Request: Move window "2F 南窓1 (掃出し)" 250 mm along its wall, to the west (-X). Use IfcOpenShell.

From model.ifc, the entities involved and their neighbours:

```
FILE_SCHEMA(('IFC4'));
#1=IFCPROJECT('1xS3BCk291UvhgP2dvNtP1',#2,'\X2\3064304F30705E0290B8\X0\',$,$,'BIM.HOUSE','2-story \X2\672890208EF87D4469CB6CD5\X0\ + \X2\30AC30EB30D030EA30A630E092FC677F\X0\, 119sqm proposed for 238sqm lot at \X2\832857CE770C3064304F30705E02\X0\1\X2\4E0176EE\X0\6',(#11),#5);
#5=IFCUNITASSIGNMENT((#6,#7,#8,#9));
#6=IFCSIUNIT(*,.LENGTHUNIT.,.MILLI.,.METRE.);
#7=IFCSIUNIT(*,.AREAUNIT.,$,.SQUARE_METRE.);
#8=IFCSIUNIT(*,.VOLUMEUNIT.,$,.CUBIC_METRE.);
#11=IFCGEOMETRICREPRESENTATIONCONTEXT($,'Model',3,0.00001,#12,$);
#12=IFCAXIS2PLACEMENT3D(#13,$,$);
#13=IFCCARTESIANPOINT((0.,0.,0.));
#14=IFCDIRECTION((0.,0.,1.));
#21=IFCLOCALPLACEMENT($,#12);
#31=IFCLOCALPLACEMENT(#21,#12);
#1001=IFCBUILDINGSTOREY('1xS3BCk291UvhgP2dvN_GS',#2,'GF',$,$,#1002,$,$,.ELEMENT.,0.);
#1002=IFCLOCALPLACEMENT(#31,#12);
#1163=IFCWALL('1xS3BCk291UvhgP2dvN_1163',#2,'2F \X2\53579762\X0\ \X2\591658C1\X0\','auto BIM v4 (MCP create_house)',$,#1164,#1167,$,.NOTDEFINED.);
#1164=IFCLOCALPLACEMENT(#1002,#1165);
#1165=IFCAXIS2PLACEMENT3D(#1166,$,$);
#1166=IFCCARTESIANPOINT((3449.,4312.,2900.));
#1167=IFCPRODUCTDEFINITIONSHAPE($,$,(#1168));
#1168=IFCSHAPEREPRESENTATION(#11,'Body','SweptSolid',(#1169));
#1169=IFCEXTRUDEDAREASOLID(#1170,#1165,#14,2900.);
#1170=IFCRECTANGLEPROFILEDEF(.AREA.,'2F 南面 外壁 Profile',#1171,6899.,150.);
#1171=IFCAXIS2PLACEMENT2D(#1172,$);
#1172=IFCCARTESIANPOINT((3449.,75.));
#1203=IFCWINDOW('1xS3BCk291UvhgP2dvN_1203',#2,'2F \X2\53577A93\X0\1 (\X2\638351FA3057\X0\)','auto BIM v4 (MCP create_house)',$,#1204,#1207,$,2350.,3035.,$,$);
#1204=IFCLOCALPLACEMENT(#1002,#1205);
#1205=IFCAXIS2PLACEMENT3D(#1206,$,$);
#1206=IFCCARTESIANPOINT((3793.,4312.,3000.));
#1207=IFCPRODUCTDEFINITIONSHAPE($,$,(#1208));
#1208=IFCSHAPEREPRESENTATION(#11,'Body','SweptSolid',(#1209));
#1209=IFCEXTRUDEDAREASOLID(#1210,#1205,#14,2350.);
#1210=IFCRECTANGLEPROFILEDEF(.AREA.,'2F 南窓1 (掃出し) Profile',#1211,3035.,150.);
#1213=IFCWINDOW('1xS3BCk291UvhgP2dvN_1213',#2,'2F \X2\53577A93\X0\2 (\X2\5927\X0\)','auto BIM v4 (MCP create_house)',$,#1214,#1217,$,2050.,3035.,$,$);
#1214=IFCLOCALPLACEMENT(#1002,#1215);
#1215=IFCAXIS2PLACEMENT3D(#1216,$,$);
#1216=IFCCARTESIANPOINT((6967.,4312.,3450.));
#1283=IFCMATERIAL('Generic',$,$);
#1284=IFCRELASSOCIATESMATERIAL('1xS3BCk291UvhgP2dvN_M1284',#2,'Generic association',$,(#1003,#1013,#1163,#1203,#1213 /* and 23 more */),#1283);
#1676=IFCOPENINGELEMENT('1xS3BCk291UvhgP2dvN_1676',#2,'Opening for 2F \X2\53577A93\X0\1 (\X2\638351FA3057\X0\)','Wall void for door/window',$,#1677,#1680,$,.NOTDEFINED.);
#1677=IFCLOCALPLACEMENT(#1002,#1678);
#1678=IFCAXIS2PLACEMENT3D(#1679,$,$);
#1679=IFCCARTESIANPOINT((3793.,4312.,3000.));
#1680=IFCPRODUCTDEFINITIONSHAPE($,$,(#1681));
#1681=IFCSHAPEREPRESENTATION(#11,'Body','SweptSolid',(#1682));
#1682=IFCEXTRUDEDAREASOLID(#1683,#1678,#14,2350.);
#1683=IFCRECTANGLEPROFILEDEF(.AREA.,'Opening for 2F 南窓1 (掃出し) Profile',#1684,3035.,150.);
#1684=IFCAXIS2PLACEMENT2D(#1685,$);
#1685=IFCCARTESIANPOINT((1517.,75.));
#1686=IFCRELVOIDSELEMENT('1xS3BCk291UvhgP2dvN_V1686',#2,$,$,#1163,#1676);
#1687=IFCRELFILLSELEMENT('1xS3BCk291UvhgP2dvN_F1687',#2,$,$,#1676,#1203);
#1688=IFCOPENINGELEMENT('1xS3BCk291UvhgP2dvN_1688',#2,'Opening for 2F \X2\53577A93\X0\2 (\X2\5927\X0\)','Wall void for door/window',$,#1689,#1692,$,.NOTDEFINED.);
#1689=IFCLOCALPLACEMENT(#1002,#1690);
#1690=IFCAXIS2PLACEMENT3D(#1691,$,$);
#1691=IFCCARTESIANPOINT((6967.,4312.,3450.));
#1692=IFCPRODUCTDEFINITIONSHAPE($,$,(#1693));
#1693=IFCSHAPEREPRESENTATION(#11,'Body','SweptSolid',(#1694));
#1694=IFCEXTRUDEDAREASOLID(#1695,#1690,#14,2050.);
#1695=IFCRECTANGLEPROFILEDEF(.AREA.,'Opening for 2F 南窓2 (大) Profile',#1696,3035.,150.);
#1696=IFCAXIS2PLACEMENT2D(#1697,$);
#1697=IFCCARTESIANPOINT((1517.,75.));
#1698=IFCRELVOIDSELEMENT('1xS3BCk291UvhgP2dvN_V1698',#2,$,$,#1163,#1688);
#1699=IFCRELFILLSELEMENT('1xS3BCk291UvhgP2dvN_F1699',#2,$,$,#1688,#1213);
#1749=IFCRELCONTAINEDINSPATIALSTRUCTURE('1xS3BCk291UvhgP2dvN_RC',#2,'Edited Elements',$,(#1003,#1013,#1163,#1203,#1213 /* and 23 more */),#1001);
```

```python
import ifcopenshell
import ifcopenshell.api.geometry
import ifcopenshell.util.placement
import ifcopenshell.util.unit

model = ifcopenshell.open("model.ifc")
unit_scale = ifcopenshell.util.unit.calculate_unit_scale(model)

window = model.by_guid("1xS3BCk291UvhgP2dvN_1203")
opening = window.FillsVoids[0].RelatingOpeningElement
wall = opening.VoidsElements[0].RelatingBuildingElement

wall_matrix = ifcopenshell.util.placement.get_local_placement(wall.ObjectPlacement)
shift = wall_matrix[:3, 0] * -0.25 / unit_scale
before = ifcopenshell.util.placement.get_local_placement(window.ObjectPlacement)[:3, 3].copy()

# The window is not placed relative to its opening, so move both.
for product in (opening, window):
    matrix = ifcopenshell.util.placement.get_local_placement(product.ObjectPlacement)
    matrix[:3, 3] += shift
    ifcopenshell.api.geometry.edit_object_placement(model, product=product, matrix=matrix, is_si=False)

after = ifcopenshell.util.placement.get_local_placement(window.ObjectPlacement)[:3, 3]
print("window moved by", (after - before).round(3) + 0.0)

model.write("model_edited.ifc")
```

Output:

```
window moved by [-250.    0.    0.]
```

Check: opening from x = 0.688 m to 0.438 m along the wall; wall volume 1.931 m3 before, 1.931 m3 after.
